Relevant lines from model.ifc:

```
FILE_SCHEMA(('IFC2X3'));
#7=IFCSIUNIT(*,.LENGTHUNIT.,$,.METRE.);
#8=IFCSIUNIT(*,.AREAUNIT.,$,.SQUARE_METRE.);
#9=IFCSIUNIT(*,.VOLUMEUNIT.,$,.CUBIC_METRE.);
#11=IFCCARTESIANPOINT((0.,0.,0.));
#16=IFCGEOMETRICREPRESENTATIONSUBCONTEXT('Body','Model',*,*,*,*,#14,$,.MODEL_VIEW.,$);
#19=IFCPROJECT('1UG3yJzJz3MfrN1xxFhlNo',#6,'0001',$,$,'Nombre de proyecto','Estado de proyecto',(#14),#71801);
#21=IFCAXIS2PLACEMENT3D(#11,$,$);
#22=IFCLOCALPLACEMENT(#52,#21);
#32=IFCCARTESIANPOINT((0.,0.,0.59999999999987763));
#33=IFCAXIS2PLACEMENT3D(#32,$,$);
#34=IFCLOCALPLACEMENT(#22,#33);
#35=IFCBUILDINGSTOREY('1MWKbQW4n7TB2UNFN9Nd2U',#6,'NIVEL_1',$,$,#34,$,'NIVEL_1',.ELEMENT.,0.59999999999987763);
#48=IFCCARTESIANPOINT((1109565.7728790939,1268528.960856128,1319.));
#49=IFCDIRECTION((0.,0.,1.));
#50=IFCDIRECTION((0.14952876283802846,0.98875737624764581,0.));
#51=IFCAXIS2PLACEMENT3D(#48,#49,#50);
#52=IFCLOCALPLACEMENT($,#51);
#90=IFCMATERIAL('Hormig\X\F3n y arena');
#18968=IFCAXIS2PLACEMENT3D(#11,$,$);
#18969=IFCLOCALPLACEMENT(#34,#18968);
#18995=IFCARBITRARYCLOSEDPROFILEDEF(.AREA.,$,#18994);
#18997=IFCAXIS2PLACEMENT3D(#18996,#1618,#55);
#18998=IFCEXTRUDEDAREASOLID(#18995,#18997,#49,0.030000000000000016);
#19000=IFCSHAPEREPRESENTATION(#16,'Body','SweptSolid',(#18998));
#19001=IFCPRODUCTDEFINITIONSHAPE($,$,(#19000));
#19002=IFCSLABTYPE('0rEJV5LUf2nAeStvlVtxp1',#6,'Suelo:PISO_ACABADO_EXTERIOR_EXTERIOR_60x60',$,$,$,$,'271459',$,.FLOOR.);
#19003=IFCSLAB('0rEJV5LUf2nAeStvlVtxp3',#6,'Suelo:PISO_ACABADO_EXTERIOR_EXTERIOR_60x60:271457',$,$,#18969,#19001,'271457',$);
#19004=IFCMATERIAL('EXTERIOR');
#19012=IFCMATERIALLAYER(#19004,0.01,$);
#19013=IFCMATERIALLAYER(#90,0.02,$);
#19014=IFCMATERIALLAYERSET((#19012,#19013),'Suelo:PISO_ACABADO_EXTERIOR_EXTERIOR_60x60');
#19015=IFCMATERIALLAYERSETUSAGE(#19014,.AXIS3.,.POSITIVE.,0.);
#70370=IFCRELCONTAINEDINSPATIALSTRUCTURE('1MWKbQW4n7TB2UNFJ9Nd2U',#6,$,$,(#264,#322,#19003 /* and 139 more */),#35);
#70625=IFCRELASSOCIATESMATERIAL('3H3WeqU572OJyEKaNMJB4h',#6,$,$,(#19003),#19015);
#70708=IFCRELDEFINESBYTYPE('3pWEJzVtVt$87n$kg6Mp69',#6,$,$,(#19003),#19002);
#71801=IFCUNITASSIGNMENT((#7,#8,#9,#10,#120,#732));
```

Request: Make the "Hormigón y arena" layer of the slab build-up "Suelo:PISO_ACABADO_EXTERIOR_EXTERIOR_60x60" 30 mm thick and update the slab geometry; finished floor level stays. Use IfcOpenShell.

```python
import ifcopenshell
import ifcopenshell.util.element
import ifcopenshell.util.representation
import ifcopenshell.util.unit

model = ifcopenshell.open("model.ifc")
unit_scale = ifcopenshell.util.unit.calculate_unit_scale(model)

layer_set = model.by_id(19014)
layer = next(l for l in layer_set.MaterialLayers if l.Material and l.Material.Name == "Hormigón y arena")
change = 0.03 / unit_scale - layer.LayerThickness
layer.LayerThickness += change

# Geometry does not follow the layer set by itself.
slabs = [e for e in ifcopenshell.util.element.get_elements_by_material(model, layer_set) if e.is_a("IfcSlab")]
for slab in sorted(slabs, key=lambda e: e.id()):
    body = ifcopenshell.util.representation.get_representation(slab, "Model", "Body")
    solid = body.Items[0]
    old_depth = solid.Depth
    solid.Depth += change
    print(slab.id(), f"{old_depth:g} -> {solid.Depth:g}")

# The layers are counted up from the underside, which has moved.
for usage in {ifcopenshell.util.element.get_material(slab) for slab in slabs}:
    usage.OffsetFromReferenceLine -= change

model.write("model_v2.ifc")
```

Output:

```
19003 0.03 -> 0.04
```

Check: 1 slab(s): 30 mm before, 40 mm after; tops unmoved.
